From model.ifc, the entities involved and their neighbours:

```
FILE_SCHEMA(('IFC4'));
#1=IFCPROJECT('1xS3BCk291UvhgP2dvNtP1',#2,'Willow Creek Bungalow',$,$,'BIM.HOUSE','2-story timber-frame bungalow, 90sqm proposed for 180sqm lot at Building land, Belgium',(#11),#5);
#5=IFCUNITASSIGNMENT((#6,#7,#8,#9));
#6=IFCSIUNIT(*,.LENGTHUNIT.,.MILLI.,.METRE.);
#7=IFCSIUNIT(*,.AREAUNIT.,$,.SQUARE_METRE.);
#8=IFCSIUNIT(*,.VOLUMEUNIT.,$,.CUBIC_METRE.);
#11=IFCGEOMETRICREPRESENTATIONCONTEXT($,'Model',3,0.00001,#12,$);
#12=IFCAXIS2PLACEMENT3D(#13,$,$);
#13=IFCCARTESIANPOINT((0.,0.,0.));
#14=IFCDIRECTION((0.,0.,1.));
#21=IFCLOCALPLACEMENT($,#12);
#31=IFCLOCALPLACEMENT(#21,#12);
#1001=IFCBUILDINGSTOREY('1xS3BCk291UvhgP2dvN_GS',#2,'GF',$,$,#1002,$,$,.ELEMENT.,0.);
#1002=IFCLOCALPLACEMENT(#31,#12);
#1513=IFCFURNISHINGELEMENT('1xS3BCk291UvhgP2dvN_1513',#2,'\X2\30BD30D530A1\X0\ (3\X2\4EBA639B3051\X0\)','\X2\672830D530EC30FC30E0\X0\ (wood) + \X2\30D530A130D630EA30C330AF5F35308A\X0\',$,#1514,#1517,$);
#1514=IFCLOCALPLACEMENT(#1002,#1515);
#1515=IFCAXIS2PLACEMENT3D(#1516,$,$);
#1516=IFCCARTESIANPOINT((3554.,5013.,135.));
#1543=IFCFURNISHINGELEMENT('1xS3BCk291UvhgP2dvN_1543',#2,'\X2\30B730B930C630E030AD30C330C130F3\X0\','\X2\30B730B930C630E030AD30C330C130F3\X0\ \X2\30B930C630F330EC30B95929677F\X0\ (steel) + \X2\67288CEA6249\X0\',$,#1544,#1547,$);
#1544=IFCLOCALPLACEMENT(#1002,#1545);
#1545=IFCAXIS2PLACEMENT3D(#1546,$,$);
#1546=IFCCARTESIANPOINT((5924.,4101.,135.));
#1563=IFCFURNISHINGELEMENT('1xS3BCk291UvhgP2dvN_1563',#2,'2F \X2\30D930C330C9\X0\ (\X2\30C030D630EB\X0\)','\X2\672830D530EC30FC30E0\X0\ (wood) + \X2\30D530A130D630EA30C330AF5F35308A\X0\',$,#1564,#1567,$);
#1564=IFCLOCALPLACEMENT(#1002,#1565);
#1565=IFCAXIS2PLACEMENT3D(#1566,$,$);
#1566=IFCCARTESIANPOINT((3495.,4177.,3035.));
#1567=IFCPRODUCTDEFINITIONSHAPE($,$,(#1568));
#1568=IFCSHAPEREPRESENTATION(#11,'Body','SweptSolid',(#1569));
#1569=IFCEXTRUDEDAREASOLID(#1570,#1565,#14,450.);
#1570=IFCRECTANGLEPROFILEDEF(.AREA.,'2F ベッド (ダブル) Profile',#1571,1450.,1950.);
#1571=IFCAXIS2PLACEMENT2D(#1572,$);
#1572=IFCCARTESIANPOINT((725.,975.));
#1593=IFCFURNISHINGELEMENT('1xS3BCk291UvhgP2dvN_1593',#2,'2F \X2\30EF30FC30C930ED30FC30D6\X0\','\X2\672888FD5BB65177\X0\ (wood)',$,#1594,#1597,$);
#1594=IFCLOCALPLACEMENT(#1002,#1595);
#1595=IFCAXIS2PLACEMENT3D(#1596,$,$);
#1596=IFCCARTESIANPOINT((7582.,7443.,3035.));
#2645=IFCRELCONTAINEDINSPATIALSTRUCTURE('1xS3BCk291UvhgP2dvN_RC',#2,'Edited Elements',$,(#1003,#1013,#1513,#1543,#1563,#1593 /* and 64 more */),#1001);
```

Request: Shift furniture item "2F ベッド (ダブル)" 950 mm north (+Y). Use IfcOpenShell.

```python
import ifcopenshell
import ifcopenshell.api.geometry
import ifcopenshell.util.placement
import ifcopenshell.util.unit

model = ifcopenshell.open("model.ifc")
unit_scale = ifcopenshell.util.unit.calculate_unit_scale(model)

item = model.by_guid("1xS3BCk291UvhgP2dvN_1563")
matrix = ifcopenshell.util.placement.get_local_placement(item.ObjectPlacement)
matrix[1, 3] += 0.95 / unit_scale
ifcopenshell.api.geometry.edit_object_placement(model, product=item, matrix=matrix, is_si=False)

print(ifcopenshell.util.placement.get_local_placement(item.ObjectPlacement).round(3) + 0.0)

model.write("model_v2.ifc")
```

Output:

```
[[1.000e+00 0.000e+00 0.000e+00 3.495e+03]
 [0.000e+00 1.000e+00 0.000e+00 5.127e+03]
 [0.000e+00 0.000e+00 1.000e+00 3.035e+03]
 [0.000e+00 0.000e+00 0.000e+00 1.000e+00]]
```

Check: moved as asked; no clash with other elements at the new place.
